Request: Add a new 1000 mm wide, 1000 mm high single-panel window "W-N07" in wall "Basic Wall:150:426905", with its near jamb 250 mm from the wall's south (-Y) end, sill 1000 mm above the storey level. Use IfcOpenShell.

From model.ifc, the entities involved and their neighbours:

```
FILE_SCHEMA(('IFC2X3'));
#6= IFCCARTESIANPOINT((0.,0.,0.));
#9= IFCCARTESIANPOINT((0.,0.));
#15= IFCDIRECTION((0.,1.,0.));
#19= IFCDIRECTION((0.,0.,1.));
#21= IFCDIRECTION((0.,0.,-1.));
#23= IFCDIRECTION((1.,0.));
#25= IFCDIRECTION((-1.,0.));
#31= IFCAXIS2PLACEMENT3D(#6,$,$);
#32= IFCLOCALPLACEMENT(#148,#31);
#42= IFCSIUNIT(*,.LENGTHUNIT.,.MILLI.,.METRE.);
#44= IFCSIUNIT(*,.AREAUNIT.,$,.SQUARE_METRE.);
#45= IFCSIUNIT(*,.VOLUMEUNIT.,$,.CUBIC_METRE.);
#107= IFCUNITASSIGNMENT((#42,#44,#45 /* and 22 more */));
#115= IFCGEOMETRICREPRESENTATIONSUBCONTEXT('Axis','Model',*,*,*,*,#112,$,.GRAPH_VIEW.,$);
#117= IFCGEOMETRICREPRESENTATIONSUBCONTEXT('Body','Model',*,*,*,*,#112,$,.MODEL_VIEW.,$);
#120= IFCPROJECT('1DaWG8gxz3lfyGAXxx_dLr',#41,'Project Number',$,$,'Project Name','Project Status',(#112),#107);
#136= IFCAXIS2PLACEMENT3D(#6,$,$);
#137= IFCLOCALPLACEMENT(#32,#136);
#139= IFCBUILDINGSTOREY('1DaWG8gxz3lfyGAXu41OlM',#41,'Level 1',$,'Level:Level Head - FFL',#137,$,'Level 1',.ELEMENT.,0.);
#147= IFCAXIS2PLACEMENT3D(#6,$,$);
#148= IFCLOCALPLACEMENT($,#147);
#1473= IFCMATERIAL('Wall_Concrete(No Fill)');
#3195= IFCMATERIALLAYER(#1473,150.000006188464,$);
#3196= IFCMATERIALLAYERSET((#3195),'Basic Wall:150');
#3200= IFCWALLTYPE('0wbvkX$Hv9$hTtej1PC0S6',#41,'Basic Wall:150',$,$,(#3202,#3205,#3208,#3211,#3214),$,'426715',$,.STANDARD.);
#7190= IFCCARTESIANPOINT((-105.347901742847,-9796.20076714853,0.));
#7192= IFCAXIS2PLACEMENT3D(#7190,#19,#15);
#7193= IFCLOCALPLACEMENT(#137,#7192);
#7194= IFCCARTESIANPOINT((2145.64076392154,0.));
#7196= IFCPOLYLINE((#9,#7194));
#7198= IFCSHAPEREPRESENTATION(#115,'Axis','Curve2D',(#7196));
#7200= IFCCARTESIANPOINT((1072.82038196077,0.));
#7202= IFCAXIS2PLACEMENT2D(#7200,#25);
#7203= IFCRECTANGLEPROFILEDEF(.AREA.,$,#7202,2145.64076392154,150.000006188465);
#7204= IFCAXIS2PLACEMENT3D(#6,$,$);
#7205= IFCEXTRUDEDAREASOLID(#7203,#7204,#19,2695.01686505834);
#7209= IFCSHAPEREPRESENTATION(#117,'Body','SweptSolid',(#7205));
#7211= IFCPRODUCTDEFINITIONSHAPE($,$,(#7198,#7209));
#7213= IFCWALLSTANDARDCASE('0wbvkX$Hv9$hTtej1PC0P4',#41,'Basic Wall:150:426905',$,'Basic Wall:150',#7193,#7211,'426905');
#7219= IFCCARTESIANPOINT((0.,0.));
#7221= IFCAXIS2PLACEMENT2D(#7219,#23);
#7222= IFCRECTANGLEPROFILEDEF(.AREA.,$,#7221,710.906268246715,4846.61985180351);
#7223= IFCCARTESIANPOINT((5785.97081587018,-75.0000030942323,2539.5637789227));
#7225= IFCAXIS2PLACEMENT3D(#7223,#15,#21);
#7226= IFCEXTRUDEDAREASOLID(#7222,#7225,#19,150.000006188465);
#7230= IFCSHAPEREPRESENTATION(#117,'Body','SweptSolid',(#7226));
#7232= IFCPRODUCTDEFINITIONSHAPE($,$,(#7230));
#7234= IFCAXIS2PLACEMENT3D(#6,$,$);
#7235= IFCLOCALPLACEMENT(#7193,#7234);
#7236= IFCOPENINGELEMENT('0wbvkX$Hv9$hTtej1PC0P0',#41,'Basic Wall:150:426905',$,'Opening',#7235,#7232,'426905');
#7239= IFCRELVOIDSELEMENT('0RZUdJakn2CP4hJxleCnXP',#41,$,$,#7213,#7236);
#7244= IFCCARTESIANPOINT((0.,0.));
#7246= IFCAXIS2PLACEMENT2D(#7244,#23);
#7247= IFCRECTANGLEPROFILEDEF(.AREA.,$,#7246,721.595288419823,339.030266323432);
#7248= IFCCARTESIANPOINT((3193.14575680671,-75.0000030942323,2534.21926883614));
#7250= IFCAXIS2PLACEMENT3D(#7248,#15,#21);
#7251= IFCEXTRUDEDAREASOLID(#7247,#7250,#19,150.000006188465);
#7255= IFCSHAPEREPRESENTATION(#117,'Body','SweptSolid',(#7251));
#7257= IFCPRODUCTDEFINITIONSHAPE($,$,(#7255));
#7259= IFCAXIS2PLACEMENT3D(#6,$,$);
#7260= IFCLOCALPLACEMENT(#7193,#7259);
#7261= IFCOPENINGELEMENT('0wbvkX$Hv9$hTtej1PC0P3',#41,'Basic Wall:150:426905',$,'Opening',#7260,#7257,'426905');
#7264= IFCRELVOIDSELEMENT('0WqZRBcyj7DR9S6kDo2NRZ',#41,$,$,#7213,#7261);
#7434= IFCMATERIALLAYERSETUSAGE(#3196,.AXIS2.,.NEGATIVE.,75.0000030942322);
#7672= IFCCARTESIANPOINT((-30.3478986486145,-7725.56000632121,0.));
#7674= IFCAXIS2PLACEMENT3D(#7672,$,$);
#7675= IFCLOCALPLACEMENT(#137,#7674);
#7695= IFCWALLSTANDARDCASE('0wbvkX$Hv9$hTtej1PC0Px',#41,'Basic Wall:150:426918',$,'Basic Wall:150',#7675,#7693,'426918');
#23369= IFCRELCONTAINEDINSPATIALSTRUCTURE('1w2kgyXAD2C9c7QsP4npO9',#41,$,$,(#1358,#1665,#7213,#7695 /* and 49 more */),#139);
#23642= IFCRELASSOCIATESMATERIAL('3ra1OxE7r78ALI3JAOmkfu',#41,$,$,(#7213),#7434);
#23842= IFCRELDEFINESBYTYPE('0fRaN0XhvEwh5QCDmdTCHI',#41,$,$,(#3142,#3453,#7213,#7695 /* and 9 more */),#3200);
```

```python
import numpy as np
import ifcopenshell
import ifcopenshell.api.feature
import ifcopenshell.api.geometry
import ifcopenshell.api.root
import ifcopenshell.api.spatial
import ifcopenshell.api.type
import ifcopenshell.geom
import ifcopenshell.util.element
import ifcopenshell.util.placement
import ifcopenshell.util.representation
import ifcopenshell.util.shape
import ifcopenshell.util.unit

model = ifcopenshell.open("model.ifc")
unit_scale = ifcopenshell.util.unit.calculate_unit_scale(model)
settings = ifcopenshell.geom.settings()


def volume(element):
    """Net volume in cubic metres, openings subtracted."""
    shape = ifcopenshell.geom.create_shape(settings, element)
    return ifcopenshell.util.shape.get_volume(shape.geometry)


wall = model.by_id(7213)
storey = ifcopenshell.util.element.get_container(wall, ifc_class="IfcBuildingStorey")
context = ifcopenshell.util.representation.get_context(model, "Model", "Body", "MODEL_VIEW")
before = volume(wall)

width, height, from_end, sill = 1, 1, 0.25, 1  # metres

# The wall runs along its own X axis, and the end named is its -X end.
wall_shape = ifcopenshell.geom.create_shape(settings, wall)
x, y, z = ifcopenshell.util.shape.get_vertices(wall_shape.geometry).T
start = x.min() + from_end
face, thickness = float(y.min()), float(y.max() - y.min())
wall_matrix = ifcopenshell.util.placement.get_local_placement(wall.ObjectPlacement)
level = ifcopenshell.util.placement.get_local_placement(storey.ObjectPlacement)[2, 3]


def in_wall(x, y):
    """Placement at x, y metres in the wall's axes, at sill height."""
    matrix = wall_matrix.copy()
    matrix[:, 3] = wall_matrix @ np.array([x / unit_scale, y / unit_scale, 0.0, 1.0])
    matrix[2, 3] = level + sill / unit_scale
    return matrix


# Opening: a box that overshoots both wall faces by 50 mm.
opening = ifcopenshell.api.root.create_entity(model, ifc_class="IfcOpeningElement")
box = ifcopenshell.api.geometry.add_wall_representation(
    model, context=context, length=width, height=height, thickness=thickness + 0.1
)
ifcopenshell.api.geometry.assign_representation(model, product=opening, representation=box)
ifcopenshell.api.geometry.edit_object_placement(model, product=opening, matrix=in_wall(start, face - 0.05), is_si=False)
ifcopenshell.api.feature.add_feature(model, feature=opening, element=wall)

window = ifcopenshell.api.root.create_entity(model, ifc_class="IfcWindow", name="W-N07")
window.OverallWidth, window.OverallHeight = width / unit_scale, height / unit_scale
body = ifcopenshell.api.geometry.add_window_representation(
    model,
    context=context,
    overall_width=window.OverallWidth,
    overall_height=window.OverallHeight,
    partition_type="SINGLE_PANEL",
)
ifcopenshell.api.geometry.assign_representation(model, product=window, representation=body)
ifcopenshell.api.spatial.assign_container(model, products=[window], relating_structure=storey)
fills = ifcopenshell.api.feature.add_filling(model, opening=opening, element=window)
fills.OwnerHistory = window.OwnerHistory  # required in IFC2X3

# IFC2X3 keeps the operation on the window style.
style = ifcopenshell.api.root.create_entity(model, ifc_class="IfcWindowStyle", name="W-N07")
style.OperationType, style.ConstructionType = "SINGLE_PANEL", "NOTDEFINED"
style.ParameterTakesPrecedence = style.Sizeable = False
ifcopenshell.api.type.assign_type(model, related_objects=[window], relating_type=style)

# Centre the window in the wall's thickness.
ifcopenshell.api.geometry.edit_object_placement(model, product=window, matrix=in_wall(start, face), is_si=False)
window_shape = ifcopenshell.geom.create_shape(settings, window)
depth = ifcopenshell.util.shape.get_vertices(window_shape.geometry)[:, 1]
offset = face + thickness / 2 - (depth.min() + depth.max()) / 2
ifcopenshell.api.geometry.edit_object_placement(model, product=window, matrix=in_wall(start, offset), is_si=False)

after = volume(wall)

print(f"wall volume {before:.3f} -> {after:.3f} m3")

model.write("model_v2.ifc")
```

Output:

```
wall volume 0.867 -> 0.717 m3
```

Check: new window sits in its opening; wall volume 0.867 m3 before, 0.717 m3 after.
